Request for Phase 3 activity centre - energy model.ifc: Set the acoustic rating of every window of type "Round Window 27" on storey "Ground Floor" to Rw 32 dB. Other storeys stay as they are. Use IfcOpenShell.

First a look at what the model holds.

```python
import ifcopenshell
import ifcopenshell.util.element

model = ifcopenshell.open("Phase 3 activity centre - energy model.ifc")
print(model.schema)
storey = next(s for s in model.by_type("IfcBuildingStorey") if s.Name == "Ground Floor")
windows = [e for e in ifcopenshell.util.element.get_decomposition(storey) if e.is_a("IfcWindow")]
seen = {}
for e in windows:
    element_type = ifcopenshell.util.element.get_type(e)
    key = (element_type.Name if element_type != e and element_type else None, ifcopenshell.util.element.get_pset(e, "Pset_WindowCommon", "AcousticRating"))
    seen[key] = seen.get(key, 0) + 1
for (name, value), count in sorted(seen.items(), key=str):
    print(count, "x", name, "|", value)
```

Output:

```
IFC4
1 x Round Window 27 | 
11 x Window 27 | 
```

```python
import ifcopenshell
import ifcopenshell.api.pset
import ifcopenshell.util.element

model = ifcopenshell.open("Phase 3 activity centre - energy model.ifc")

storey = next(s for s in model.by_type("IfcBuildingStorey") if s.Name == "Ground Floor")
windows = [e for e in ifcopenshell.util.element.get_decomposition(storey) if e.is_a("IfcWindow")]

count = 0
for e in windows:
    element_type = ifcopenshell.util.element.get_type(e)
    if element_type in (None, e) or element_type.Name != "Round Window 27":
        continue
    # add_pset returns the element's existing set when there is one.
    pset = ifcopenshell.api.pset.add_pset(model, product=e, name="Pset_WindowCommon")
    ifcopenshell.api.pset.edit_pset(model, pset=pset, properties={"AcousticRating": "Rw 32 dB"})
    count += 1

print(count, "windows updated")

model.write("Phase 3 activity centre - energy model-out.ifc")
```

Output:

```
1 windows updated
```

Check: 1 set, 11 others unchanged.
